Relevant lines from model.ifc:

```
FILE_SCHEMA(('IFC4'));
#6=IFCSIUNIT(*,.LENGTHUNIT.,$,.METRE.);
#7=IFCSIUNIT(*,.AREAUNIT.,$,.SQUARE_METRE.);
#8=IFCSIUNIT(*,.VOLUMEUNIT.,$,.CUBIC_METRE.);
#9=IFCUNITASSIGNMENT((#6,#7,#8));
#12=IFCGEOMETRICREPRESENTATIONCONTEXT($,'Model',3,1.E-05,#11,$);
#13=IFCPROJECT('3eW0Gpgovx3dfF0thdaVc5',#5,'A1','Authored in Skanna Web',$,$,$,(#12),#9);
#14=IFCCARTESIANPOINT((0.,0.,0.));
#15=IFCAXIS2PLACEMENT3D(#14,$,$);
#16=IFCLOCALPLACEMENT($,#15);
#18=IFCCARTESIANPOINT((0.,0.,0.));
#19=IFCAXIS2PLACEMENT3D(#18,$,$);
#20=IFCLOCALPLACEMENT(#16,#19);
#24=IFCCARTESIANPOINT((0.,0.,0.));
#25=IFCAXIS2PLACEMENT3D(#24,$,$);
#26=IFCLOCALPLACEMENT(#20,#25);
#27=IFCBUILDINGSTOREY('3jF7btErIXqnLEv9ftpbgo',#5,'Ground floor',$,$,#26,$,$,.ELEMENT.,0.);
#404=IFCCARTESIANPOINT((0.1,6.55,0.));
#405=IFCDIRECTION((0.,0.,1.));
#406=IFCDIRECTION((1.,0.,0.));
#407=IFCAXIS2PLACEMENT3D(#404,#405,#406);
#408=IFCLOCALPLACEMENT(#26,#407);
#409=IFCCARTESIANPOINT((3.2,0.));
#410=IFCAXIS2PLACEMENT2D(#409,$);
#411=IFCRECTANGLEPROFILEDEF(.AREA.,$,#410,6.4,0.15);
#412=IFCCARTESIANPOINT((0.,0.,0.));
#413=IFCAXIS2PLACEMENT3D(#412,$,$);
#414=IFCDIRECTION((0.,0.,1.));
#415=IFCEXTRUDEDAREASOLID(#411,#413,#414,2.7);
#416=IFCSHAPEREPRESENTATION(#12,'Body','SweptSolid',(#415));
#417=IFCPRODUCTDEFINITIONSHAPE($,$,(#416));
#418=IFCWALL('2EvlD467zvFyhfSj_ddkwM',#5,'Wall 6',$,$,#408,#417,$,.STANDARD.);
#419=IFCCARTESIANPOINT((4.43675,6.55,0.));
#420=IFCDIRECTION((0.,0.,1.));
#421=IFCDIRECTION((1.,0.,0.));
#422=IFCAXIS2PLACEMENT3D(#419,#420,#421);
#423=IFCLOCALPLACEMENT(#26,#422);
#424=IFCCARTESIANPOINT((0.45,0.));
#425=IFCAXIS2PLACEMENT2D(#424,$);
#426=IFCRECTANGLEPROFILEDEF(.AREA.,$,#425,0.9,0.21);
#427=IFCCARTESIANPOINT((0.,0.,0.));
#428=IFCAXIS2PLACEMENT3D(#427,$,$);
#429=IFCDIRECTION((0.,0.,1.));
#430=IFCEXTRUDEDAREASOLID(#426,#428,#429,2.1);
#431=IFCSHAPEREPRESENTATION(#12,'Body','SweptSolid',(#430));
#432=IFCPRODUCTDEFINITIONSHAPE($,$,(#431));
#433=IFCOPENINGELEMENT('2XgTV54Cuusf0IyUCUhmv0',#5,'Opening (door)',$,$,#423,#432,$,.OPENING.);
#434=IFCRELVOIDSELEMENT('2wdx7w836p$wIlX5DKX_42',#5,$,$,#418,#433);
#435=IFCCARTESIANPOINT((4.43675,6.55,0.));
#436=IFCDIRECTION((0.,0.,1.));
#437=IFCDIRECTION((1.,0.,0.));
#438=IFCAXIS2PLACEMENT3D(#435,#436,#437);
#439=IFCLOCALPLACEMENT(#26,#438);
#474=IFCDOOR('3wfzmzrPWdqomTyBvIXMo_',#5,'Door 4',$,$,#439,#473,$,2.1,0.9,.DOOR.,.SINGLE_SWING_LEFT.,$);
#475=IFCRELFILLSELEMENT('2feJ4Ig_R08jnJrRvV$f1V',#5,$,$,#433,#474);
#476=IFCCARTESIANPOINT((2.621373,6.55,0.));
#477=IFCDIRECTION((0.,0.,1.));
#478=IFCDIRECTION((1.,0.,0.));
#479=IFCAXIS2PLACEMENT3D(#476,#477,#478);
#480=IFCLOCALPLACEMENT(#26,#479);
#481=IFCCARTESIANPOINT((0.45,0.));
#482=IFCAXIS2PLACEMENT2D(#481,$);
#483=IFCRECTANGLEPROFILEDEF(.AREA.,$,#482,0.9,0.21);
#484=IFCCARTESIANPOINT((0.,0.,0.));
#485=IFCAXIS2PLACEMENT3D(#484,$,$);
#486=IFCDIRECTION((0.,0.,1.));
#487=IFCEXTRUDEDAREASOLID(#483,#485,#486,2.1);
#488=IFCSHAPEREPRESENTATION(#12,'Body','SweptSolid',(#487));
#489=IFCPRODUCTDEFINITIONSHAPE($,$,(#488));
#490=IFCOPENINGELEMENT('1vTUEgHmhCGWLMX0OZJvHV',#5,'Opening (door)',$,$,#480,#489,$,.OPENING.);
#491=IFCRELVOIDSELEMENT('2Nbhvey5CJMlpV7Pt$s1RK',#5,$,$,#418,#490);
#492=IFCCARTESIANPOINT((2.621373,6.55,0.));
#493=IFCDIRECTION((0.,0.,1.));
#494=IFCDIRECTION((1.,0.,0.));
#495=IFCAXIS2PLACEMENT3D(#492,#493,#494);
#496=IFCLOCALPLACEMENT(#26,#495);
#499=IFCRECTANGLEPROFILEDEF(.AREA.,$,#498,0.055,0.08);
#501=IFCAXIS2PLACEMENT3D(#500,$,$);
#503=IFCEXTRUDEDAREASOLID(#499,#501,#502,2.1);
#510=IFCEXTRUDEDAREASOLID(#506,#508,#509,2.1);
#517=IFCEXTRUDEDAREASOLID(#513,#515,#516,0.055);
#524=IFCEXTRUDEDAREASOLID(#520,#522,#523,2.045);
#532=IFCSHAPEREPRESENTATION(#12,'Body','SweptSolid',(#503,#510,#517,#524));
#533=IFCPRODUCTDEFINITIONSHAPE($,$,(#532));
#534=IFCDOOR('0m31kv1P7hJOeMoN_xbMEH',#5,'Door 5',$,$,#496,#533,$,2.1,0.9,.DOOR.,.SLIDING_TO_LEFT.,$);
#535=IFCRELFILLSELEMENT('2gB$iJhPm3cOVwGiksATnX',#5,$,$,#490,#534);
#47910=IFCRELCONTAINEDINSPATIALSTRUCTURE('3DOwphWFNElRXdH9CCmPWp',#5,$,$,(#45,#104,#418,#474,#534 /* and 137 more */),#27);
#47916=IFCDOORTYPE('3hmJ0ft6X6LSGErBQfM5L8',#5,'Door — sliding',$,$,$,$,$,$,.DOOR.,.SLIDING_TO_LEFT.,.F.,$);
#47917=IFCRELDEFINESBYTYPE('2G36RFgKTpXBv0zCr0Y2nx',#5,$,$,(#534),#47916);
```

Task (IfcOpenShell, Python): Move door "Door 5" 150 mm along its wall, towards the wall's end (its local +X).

```python
import ifcopenshell
import ifcopenshell.api.geometry
import ifcopenshell.util.placement
import ifcopenshell.util.unit

model = ifcopenshell.open("model.ifc")
unit_scale = ifcopenshell.util.unit.calculate_unit_scale(model)

door = model.by_guid("0m31kv1P7hJOeMoN_xbMEH")
opening = door.FillsVoids[0].RelatingOpeningElement
wall = opening.VoidsElements[0].RelatingBuildingElement

wall_matrix = ifcopenshell.util.placement.get_local_placement(wall.ObjectPlacement)
shift = wall_matrix[:3, 0] * 0.15 / unit_scale
before = ifcopenshell.util.placement.get_local_placement(door.ObjectPlacement)[:3, 3].copy()

# The door is not placed relative to its opening, so move both.
for product in (opening, door):
    matrix = ifcopenshell.util.placement.get_local_placement(product.ObjectPlacement)
    matrix[:3, 3] += shift
    ifcopenshell.api.geometry.edit_object_placement(model, product=product, matrix=matrix, is_si=False)

after = ifcopenshell.util.placement.get_local_placement(door.ObjectPlacement)[:3, 3]
print("door moved by", (after - before).round(3) + 0.0)

model.write("model-out.ifc")
```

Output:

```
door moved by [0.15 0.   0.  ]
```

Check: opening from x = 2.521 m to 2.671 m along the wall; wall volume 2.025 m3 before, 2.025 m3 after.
